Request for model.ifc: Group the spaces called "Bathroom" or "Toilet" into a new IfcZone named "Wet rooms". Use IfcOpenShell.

First a look at what the model holds.

```python
import ifcopenshell

model = ifcopenshell.open("model.ifc")
print(model.schema)
seen = {}
for space in model.by_type("IfcSpace"):
    seen[space.LongName] = seen.get(space.LongName, 0) + 1
for name, count in sorted(seen.items(), key=str):
    print(count, "x", name)
print("zones:", [z.Name for z in model.by_type("IfcZone")][:20])
```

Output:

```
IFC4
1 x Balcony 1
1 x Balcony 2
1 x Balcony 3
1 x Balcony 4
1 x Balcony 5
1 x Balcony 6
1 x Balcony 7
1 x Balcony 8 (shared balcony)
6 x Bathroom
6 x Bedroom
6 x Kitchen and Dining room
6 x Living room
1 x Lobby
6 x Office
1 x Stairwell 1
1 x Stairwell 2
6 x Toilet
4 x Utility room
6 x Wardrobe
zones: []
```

```python
import ifcopenshell
import ifcopenshell.api.group
import ifcopenshell.api.root

model = ifcopenshell.open("model.ifc")

names = {"Bathroom", "Toilet"}
spaces = [s for s in model.by_type("IfcSpace") if s.LongName in names]

zone = ifcopenshell.api.root.create_entity(model, ifc_class="IfcZone", name="Wet rooms")
ifcopenshell.api.group.assign_group(model, products=spaces, group=zone)
print(len(spaces), "spaces in", zone.Name)

model.write("model_edited.ifc")
```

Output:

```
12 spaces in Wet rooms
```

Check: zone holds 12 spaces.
